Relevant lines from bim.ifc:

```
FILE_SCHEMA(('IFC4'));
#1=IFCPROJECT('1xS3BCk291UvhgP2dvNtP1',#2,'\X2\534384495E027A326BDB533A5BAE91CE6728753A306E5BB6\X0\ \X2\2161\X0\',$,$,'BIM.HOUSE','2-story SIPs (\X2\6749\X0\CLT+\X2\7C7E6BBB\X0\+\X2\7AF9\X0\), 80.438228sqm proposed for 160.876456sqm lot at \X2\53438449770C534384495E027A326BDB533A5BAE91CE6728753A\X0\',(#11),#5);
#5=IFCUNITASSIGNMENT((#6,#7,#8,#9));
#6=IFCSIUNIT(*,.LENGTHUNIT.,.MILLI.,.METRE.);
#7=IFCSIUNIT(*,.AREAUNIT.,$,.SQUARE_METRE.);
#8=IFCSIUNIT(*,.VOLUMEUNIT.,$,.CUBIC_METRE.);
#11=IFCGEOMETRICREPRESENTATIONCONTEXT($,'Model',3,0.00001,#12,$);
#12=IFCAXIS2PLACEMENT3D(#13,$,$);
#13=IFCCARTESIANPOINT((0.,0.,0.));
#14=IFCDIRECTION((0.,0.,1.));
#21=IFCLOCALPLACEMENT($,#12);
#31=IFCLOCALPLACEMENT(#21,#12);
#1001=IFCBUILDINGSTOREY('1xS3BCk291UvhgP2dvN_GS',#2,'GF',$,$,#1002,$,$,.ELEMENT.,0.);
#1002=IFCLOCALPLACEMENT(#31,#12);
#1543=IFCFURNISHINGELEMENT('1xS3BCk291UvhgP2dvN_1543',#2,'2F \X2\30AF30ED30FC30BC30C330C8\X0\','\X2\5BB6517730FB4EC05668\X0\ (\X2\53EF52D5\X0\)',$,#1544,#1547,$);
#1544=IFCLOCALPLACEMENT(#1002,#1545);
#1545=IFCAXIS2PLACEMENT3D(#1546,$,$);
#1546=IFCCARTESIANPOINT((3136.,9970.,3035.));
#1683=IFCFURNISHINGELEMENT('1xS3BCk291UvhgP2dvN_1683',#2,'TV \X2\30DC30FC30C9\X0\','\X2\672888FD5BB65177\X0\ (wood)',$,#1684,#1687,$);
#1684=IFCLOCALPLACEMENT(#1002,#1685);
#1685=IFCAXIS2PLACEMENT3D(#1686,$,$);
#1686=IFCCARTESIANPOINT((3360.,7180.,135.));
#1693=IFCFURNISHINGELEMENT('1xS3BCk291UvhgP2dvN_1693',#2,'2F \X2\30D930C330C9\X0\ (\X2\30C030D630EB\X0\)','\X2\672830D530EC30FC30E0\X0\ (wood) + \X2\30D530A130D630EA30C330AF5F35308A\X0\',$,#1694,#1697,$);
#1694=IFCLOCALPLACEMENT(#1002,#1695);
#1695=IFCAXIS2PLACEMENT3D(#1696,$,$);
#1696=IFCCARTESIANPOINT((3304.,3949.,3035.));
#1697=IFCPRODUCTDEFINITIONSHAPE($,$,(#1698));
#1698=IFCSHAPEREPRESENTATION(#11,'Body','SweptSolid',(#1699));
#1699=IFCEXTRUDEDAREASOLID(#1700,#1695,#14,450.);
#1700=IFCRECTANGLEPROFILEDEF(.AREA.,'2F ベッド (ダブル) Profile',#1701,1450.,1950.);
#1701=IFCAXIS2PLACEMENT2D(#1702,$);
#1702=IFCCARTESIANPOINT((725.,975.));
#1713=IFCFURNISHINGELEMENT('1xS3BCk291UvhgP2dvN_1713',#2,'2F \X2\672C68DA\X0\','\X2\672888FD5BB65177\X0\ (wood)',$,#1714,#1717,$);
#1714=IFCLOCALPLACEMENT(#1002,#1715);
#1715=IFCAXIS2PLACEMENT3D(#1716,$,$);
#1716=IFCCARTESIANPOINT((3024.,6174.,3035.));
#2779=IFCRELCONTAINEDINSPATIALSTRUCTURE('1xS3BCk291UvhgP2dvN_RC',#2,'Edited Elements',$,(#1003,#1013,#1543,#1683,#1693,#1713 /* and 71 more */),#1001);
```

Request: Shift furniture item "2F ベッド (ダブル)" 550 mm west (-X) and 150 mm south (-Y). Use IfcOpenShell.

```python
import ifcopenshell
import ifcopenshell.api.geometry
import ifcopenshell.util.placement

model = ifcopenshell.open("bim.ifc")

item = model.by_guid("1xS3BCk291UvhgP2dvN_1693")
matrix = ifcopenshell.util.placement.get_local_placement(item.ObjectPlacement)
matrix[0, 3] -= 550.0
matrix[1, 3] -= 150.0
ifcopenshell.api.geometry.edit_object_placement(model, product=item, matrix=matrix, is_si=False)

print(ifcopenshell.util.placement.get_local_placement(item.ObjectPlacement).round(3) + 0.0)

model.write("bim_v2.ifc")
```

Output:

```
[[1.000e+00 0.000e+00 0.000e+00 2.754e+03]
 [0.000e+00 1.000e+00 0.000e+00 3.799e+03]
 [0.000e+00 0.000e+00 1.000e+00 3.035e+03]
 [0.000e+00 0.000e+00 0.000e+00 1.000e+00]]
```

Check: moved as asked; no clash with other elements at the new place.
